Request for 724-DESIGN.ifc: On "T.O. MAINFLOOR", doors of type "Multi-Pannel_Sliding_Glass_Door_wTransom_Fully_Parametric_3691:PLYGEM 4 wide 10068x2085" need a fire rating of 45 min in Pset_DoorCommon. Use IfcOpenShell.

First a look at what the model holds.

```python
import ifcopenshell
import ifcopenshell.util.element

model = ifcopenshell.open("724-DESIGN.ifc")
print(model.schema)
storey = next(s for s in model.by_type("IfcBuildingStorey") if s.Name == "T.O. MAINFLOOR")
doors = [e for e in ifcopenshell.util.element.get_decomposition(storey) if e.is_a("IfcDoor")]
seen = {}
for e in doors:
    element_type = ifcopenshell.util.element.get_type(e)
    key = (element_type.Name if element_type != e and element_type else None, ifcopenshell.util.element.get_pset(e, "Pset_DoorCommon", "FireRating"))
    seen[key] = seen.get(key, 0) + 1
for (name, value), count in sorted(seen.items(), key=str):
    print(count, "x", name, "|", value)
```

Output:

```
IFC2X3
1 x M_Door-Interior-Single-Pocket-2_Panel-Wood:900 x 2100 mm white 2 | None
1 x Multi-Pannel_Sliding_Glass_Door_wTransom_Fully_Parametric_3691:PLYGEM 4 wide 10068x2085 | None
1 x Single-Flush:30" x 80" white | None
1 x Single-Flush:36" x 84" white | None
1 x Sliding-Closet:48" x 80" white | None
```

```python
import ifcopenshell
import ifcopenshell.api.pset
import ifcopenshell.util.element

model = ifcopenshell.open("724-DESIGN.ifc")

storey = next(s for s in model.by_type("IfcBuildingStorey") if s.Name == "T.O. MAINFLOOR")
doors = [e for e in ifcopenshell.util.element.get_decomposition(storey) if e.is_a("IfcDoor")]

count = 0
for e in doors:
    element_type = ifcopenshell.util.element.get_type(e)
    if element_type in (None, e) or element_type.Name != "Multi-Pannel_Sliding_Glass_Door_wTransom_Fully_Parametric_3691:PLYGEM 4 wide 10068x2085":
        continue
    # add_pset returns the element's existing set when there is one.
    pset = ifcopenshell.api.pset.add_pset(model, product=e, name="Pset_DoorCommon")
    ifcopenshell.api.pset.edit_pset(model, pset=pset, properties={"FireRating": "45 min"})
    count += 1

print(count, "doors updated")

model.write("724-DESIGN-out.ifc")
```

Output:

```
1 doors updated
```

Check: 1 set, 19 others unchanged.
